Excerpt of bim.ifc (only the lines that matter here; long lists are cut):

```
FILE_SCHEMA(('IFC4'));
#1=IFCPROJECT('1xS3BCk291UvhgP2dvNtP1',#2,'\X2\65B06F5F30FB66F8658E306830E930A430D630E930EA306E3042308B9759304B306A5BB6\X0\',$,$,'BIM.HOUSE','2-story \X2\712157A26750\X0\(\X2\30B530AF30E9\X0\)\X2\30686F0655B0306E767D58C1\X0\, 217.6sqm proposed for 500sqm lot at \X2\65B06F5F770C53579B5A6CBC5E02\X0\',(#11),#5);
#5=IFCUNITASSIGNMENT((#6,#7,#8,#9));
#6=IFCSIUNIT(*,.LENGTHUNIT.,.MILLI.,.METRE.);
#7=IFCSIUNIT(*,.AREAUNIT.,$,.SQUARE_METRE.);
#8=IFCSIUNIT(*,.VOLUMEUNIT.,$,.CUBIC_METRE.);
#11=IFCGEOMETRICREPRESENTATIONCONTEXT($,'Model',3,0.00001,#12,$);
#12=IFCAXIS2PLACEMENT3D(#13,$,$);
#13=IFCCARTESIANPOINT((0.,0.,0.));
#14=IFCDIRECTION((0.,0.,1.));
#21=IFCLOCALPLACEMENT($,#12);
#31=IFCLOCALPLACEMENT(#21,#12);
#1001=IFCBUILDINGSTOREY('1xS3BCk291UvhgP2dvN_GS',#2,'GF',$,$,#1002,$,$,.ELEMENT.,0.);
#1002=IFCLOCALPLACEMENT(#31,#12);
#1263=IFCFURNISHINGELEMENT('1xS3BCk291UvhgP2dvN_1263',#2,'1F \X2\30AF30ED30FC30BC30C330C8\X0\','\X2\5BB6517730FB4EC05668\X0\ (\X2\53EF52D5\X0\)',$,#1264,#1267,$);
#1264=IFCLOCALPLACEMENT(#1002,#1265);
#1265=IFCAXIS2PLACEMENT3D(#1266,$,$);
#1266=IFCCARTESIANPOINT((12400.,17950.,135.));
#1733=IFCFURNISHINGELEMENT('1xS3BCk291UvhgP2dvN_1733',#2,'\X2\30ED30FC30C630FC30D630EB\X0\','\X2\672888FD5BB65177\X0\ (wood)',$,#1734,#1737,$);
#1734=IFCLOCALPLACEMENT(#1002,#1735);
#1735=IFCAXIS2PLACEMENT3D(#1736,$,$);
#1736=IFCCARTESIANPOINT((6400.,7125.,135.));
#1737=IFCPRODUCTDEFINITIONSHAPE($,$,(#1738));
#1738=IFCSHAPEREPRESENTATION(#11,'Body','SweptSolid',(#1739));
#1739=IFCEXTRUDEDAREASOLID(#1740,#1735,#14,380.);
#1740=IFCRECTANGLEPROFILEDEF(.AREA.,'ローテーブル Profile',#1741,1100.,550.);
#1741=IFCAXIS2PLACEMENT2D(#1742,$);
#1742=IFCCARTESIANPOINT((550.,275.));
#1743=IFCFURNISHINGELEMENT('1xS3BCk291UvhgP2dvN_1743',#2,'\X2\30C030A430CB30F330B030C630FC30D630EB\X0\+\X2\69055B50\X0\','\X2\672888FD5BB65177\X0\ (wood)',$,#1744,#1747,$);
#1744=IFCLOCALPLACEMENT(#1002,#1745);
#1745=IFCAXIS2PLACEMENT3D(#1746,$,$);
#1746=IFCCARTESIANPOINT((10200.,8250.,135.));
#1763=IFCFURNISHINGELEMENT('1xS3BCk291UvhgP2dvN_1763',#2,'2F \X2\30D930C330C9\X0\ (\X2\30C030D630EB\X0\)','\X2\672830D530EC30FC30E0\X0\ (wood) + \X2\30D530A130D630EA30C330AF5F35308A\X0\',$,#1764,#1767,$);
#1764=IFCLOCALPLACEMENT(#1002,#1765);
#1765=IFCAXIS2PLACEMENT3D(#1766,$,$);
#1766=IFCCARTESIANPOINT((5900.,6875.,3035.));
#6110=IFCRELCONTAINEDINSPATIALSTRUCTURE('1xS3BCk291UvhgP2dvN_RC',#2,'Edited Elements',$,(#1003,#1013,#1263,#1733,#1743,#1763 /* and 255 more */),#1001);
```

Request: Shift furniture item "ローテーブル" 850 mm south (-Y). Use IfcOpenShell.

```python
import ifcopenshell
import ifcopenshell.api.geometry
import ifcopenshell.util.placement
import ifcopenshell.util.unit

model = ifcopenshell.open("bim.ifc")
unit_scale = ifcopenshell.util.unit.calculate_unit_scale(model)

item = model.by_guid("1xS3BCk291UvhgP2dvN_1733")
matrix = ifcopenshell.util.placement.get_local_placement(item.ObjectPlacement)
matrix[1, 3] -= 0.85 / unit_scale
ifcopenshell.api.geometry.edit_object_placement(model, product=item, matrix=matrix, is_si=False)

print(ifcopenshell.util.placement.get_local_placement(item.ObjectPlacement).round(3) + 0.0)

model.write("bim_edited.ifc")
```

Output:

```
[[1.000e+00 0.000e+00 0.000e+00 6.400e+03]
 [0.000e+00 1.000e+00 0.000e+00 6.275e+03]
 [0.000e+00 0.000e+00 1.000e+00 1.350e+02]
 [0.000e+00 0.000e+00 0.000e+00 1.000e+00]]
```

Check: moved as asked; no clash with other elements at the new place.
